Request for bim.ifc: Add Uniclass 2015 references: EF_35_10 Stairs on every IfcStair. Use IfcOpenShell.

First a look at what the model holds.

```python
import ifcopenshell

model = ifcopenshell.open("bim.ifc")
print(model.schema)
print("classifications:", [c.Name for c in model.by_type("IfcClassification")])
for ifc_class in ("IfcDoor", "IfcRoof", "IfcStair", "IfcWall", "IfcWindow"):
    print(ifc_class, len(model.by_type(ifc_class)))
```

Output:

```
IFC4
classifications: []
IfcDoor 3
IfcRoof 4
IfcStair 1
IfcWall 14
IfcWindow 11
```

```python
import ifcopenshell
import ifcopenshell.api.classification

model = ifcopenshell.open("bim.ifc")

system = ifcopenshell.api.classification.add_classification(model, classification="Uniclass 2015")

codes = {
    "IfcStair": ("EF_35_10", "Stairs"),
}
for ifc_class, (code, name) in codes.items():
    products = model.by_type(ifc_class)
    ifcopenshell.api.classification.add_reference(
        model, products=products, classification=system, identification=code, name=name
    )
    print(code, len(products))

model.write("bim_rev.ifc")
```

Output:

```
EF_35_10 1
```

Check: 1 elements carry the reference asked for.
